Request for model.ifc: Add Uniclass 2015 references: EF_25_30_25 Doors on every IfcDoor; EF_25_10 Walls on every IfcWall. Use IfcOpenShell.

First a look at what the model holds.

```python
import ifcopenshell

model = ifcopenshell.open("model.ifc")
print(model.schema)
print("classifications:", [c.Name for c in model.by_type("IfcClassification")])
for ifc_class in ("IfcDoor", "IfcRoof", "IfcStair", "IfcWall", "IfcWindow"):
    print(ifc_class, len(model.by_type(ifc_class)))
```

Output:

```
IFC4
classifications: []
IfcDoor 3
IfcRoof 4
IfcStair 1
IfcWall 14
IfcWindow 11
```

```python
import ifcopenshell
import ifcopenshell.api.classification

model = ifcopenshell.open("model.ifc")

system = ifcopenshell.api.classification.add_classification(model, classification="Uniclass 2015")

codes = {
    "IfcDoor": ("EF_25_30_25", "Doors"),
    "IfcWall": ("EF_25_10", "Walls"),
}
for ifc_class, (code, name) in codes.items():
    products = model.by_type(ifc_class)
    ifcopenshell.api.classification.add_reference(
        model, products=products, classification=system, identification=code, name=name
    )
    print(code, len(products))

model.write("model_updated.ifc")
```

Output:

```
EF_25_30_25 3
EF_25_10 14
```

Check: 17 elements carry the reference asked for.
